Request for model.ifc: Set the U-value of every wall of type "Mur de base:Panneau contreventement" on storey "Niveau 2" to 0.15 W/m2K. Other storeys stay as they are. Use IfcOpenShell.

First a look at what the model holds.

```python
import ifcopenshell
import ifcopenshell.util.element

model = ifcopenshell.open("model.ifc")
print(model.schema)
storey = next(s for s in model.by_type("IfcBuildingStorey") if s.Name == "Niveau 2")
walls = [e for e in ifcopenshell.util.element.get_decomposition(storey) if e.is_a("IfcWall")]
seen = {}
for e in walls:
    element_type = ifcopenshell.util.element.get_type(e)
    key = (element_type.Name if element_type != e and element_type else None, ifcopenshell.util.element.get_pset(e, "Pset_WallCommon", "ThermalTransmittance"))
    seen[key] = seen.get(key, 0) + 1
for (name, value), count in sorted(seen.items(), key=str):
    print(count, "x", name, "|", value)
```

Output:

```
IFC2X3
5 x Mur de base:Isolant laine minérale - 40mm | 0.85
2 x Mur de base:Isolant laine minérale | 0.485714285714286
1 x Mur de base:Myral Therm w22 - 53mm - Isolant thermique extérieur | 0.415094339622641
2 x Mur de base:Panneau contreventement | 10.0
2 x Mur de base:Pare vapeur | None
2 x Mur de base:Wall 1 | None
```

```python
import ifcopenshell
import ifcopenshell.api.pset
import ifcopenshell.util.element

model = ifcopenshell.open("model.ifc")

storey = next(s for s in model.by_type("IfcBuildingStorey") if s.Name == "Niveau 2")
walls = [e for e in ifcopenshell.util.element.get_decomposition(storey) if e.is_a("IfcWall")]

count = 0
for e in walls:
    element_type = ifcopenshell.util.element.get_type(e)
    if element_type in (None, e) or element_type.Name != "Mur de base:Panneau contreventement":
        continue
    # add_pset returns the element's existing set when there is one.
    pset = ifcopenshell.api.pset.add_pset(model, product=e, name="Pset_WallCommon")
    ifcopenshell.api.pset.edit_pset(model, pset=pset, properties={"ThermalTransmittance": 0.15})
    count += 1

print(count, "walls updated")

model.write("model_edited.ifc")
```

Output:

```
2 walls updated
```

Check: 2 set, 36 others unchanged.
